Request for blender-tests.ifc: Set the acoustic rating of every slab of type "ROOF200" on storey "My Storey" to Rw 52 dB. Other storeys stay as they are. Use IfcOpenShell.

First a look at what the model holds.

```python
import ifcopenshell
import ifcopenshell.util.element

model = ifcopenshell.open("blender-tests.ifc")
print(model.schema)
storey = next(s for s in model.by_type("IfcBuildingStorey") if s.Name == "My Storey")
slabs = [e for e in ifcopenshell.util.element.get_decomposition(storey) if e.is_a("IfcSlab")]
seen = {}
for e in slabs:
    element_type = ifcopenshell.util.element.get_type(e)
    key = (element_type.Name if element_type != e and element_type else None, ifcopenshell.util.element.get_pset(e, "Pset_SlabCommon", "AcousticRating"))
    seen[key] = seen.get(key, 0) + 1
for (name, value), count in sorted(seen.items(), key=str):
    print(count, "x", name, "|", value)
```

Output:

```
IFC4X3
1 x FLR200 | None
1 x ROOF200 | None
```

```python
import ifcopenshell
import ifcopenshell.api.pset
import ifcopenshell.util.element

model = ifcopenshell.open("blender-tests.ifc")

storey = next(s for s in model.by_type("IfcBuildingStorey") if s.Name == "My Storey")
slabs = [e for e in ifcopenshell.util.element.get_decomposition(storey) if e.is_a("IfcSlab")]

count = 0
for e in slabs:
    element_type = ifcopenshell.util.element.get_type(e)
    if element_type in (None, e) or element_type.Name != "ROOF200":
        continue
    # add_pset returns the element's existing set when there is one.
    pset = ifcopenshell.api.pset.add_pset(model, product=e, name="Pset_SlabCommon")
    ifcopenshell.api.pset.edit_pset(model, pset=pset, properties={"AcousticRating": "Rw 52 dB"})
    count += 1

print(count, "slabs updated")

model.write("blender-tests_updated.ifc")
```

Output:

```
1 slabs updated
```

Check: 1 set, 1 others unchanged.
